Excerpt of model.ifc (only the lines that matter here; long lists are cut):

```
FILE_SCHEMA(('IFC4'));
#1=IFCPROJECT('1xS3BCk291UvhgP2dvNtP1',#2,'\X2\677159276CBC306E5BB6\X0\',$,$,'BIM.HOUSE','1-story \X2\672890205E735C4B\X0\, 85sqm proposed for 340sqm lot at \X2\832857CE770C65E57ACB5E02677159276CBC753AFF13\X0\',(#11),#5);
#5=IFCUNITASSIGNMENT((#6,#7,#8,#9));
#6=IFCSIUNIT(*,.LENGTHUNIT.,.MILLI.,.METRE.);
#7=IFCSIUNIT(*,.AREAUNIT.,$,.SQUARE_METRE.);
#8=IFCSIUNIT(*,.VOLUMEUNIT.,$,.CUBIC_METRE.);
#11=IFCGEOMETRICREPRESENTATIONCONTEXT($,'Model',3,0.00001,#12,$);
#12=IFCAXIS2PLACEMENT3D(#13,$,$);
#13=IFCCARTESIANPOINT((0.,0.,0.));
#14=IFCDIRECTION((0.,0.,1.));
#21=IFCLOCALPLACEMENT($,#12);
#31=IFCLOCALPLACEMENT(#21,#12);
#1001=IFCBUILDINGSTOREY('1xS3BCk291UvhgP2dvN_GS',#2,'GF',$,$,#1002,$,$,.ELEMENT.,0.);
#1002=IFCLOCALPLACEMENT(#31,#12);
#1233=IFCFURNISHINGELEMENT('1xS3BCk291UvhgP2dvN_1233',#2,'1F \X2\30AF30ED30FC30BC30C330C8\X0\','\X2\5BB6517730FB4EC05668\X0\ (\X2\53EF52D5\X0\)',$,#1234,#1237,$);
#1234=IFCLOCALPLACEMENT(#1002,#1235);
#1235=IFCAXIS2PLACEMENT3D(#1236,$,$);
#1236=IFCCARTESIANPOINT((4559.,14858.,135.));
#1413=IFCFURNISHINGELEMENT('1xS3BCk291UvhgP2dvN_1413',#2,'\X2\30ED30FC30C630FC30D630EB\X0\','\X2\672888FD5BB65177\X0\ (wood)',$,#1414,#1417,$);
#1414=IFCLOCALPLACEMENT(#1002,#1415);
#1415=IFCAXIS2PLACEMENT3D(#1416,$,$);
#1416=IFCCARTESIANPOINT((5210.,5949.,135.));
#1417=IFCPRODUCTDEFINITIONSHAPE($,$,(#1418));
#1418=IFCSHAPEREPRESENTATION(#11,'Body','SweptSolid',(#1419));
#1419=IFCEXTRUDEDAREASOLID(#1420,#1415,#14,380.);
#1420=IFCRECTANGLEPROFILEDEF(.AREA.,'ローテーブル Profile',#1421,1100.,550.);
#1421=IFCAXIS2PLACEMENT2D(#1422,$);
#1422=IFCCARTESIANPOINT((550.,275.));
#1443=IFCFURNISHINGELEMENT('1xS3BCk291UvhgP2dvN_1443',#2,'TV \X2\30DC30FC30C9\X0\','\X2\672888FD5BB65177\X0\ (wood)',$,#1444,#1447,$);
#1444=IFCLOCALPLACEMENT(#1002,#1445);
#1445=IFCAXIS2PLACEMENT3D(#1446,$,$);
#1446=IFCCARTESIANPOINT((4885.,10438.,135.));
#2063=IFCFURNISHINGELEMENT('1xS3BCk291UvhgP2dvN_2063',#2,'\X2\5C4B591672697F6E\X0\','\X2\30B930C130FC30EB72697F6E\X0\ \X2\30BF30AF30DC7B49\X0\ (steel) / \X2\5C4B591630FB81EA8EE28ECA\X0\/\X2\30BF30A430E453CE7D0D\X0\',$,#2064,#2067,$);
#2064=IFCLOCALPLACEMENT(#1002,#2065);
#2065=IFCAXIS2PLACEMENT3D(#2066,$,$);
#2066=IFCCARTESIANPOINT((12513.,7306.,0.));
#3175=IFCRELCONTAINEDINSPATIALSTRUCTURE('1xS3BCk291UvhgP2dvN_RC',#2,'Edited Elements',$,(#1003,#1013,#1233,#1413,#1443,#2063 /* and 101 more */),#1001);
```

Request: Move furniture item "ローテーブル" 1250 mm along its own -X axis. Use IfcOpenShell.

```python
import ifcopenshell
import ifcopenshell.api.geometry
import ifcopenshell.util.placement

model = ifcopenshell.open("model.ifc")

item = model.by_guid("1xS3BCk291UvhgP2dvN_1413")
matrix = ifcopenshell.util.placement.get_local_placement(item.ObjectPlacement)
matrix[:3, 3] -= matrix[:3, 0] * 1250.0
ifcopenshell.api.geometry.edit_object_placement(model, product=item, matrix=matrix, is_si=False)

print(ifcopenshell.util.placement.get_local_placement(item.ObjectPlacement).round(3) + 0.0)

model.write("model_edited.ifc")
```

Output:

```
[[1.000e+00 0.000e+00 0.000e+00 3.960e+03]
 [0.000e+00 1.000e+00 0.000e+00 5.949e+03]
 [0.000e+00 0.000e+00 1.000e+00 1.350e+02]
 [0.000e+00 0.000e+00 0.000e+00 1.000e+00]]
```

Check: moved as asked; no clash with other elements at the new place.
